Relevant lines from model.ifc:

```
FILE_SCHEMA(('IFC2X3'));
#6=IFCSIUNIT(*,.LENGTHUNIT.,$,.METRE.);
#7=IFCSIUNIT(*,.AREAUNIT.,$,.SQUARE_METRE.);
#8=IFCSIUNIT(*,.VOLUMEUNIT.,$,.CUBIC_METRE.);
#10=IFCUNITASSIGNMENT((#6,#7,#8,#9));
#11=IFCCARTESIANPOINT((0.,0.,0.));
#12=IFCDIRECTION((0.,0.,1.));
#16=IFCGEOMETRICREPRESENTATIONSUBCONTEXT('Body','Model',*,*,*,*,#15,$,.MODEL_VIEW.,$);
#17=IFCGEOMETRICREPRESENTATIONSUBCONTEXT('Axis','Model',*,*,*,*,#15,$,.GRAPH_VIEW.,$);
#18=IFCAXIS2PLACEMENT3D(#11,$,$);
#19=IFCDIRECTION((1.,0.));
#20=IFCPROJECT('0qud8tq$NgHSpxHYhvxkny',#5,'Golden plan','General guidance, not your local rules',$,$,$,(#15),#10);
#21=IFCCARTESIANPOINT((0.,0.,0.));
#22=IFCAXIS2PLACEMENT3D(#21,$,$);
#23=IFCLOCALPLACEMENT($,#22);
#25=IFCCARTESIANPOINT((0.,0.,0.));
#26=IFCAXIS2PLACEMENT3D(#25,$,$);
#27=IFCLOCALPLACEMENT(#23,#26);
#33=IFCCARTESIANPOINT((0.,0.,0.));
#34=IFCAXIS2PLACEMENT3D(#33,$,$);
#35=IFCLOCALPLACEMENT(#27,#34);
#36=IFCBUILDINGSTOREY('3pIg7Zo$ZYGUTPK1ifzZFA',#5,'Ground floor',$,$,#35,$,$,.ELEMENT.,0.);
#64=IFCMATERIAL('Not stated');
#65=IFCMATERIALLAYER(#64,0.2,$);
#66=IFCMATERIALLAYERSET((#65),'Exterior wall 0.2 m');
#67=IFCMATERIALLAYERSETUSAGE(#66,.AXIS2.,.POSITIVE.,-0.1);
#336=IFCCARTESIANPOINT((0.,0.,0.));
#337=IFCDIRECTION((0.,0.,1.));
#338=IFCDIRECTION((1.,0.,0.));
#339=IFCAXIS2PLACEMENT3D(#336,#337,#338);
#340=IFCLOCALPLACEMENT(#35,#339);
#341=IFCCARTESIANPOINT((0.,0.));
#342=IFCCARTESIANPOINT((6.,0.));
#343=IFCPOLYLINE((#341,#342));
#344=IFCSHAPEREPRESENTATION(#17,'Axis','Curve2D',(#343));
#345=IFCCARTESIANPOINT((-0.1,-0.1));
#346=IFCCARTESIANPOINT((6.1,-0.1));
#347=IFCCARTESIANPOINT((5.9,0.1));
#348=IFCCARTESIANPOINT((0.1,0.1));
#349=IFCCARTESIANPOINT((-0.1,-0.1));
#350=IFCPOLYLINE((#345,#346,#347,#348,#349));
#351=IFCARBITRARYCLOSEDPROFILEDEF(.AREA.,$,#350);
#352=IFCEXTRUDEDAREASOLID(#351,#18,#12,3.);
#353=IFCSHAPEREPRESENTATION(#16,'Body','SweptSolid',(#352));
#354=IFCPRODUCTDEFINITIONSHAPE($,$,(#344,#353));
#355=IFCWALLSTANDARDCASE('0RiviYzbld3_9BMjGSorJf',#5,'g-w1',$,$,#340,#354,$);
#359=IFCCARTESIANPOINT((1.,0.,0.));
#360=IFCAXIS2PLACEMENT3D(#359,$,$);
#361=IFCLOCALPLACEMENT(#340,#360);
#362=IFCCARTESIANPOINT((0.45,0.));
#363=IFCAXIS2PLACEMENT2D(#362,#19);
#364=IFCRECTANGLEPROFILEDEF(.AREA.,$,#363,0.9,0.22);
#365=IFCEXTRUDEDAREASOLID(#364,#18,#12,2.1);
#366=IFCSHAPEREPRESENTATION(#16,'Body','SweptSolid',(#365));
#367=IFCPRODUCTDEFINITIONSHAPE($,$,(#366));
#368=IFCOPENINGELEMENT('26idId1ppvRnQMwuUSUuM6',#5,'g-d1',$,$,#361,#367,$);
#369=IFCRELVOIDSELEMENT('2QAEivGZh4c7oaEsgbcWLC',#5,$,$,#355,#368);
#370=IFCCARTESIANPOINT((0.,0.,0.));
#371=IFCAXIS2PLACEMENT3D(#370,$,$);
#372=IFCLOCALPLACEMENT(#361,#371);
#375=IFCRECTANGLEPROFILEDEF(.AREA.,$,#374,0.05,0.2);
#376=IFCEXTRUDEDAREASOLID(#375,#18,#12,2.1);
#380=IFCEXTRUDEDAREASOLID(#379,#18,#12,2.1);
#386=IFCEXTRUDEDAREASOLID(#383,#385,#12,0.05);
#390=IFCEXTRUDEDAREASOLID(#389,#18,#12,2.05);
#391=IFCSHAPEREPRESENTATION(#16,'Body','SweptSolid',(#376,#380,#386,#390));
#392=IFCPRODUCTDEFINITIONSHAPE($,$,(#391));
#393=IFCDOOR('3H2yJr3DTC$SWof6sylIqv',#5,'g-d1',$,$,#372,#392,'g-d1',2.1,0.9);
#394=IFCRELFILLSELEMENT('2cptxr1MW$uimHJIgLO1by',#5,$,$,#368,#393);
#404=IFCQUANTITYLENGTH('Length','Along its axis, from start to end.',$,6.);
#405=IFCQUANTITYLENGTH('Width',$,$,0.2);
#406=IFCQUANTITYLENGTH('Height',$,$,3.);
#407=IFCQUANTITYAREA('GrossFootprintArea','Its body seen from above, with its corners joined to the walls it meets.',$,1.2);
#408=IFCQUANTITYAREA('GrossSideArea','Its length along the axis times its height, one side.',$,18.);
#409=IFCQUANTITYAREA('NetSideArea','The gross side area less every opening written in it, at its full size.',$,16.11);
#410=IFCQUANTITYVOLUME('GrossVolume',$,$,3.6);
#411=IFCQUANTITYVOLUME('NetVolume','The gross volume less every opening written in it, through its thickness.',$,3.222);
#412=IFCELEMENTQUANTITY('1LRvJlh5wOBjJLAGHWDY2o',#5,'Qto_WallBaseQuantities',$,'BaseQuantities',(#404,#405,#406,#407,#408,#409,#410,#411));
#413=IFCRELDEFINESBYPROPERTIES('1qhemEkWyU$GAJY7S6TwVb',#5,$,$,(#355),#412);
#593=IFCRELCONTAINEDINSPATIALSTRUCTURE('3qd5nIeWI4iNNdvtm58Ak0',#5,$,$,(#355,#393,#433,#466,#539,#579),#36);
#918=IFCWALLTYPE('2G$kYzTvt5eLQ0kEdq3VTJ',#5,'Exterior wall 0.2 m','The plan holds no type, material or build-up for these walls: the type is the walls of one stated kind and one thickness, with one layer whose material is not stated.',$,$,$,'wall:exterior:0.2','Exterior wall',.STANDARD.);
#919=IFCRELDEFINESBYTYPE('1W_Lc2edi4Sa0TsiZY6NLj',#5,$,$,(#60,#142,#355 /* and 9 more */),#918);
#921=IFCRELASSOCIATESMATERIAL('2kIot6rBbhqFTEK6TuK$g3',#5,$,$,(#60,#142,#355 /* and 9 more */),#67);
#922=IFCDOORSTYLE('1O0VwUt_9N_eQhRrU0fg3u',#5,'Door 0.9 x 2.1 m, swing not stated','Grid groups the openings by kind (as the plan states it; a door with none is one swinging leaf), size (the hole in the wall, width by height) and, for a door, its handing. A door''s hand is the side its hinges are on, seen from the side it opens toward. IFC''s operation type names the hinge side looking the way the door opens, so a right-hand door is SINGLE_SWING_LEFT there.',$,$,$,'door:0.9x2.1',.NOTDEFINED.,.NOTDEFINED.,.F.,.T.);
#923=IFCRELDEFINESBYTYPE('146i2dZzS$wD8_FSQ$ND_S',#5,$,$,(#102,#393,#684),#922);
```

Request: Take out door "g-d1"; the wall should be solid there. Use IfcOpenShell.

```python
import ifcopenshell
import ifcopenshell.api.feature
import ifcopenshell.api.pset
import ifcopenshell.api.root
import ifcopenshell.geom
import ifcopenshell.util.element
import ifcopenshell.util.shape
import ifcopenshell.util.unit

model = ifcopenshell.open("model.ifc")
area_scale = ifcopenshell.util.unit.calculate_unit_scale(model, "AREAUNIT")
volume_scale = ifcopenshell.util.unit.calculate_unit_scale(model, "VOLUMEUNIT")
settings = ifcopenshell.geom.settings()


def volume(element):
    """Net volume in cubic metres, openings subtracted."""
    shape = ifcopenshell.geom.create_shape(settings, element)
    return ifcopenshell.util.shape.get_volume(shape.geometry)


door = model.by_guid("3H2yJr3DTC$SWof6sylIqv")
opening = door.FillsVoids[0].RelatingOpeningElement
wall = opening.VoidsElements[0].RelatingBuildingElement
before = volume(wall)

ifcopenshell.api.root.remove_product(model, product=door)
ifcopenshell.api.feature.remove_feature(model, feature=opening)

after = volume(wall)
thickness = 0.2  # wall thickness in metres

# Update the wall's stored quantities.
qto = model.by_id(ifcopenshell.util.element.get_pset(wall, "Qto_WallBaseQuantities", should_inherit=False)["id"])
ifcopenshell.api.pset.edit_qto(model, qto=qto, properties={
    "NetSideArea": after / thickness / area_scale,
    "NetVolume": after / volume_scale,
})

print(f"wall volume {before:.3f} -> {after:.3f} m3")

model.write("model_updated.ifc")
```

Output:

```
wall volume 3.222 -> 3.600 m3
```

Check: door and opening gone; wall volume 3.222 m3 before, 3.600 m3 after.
